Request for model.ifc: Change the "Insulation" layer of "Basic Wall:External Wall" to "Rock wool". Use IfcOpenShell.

First a look at what the model holds.

```python
import ifcopenshell
import ifcopenshell.util.element

model = ifcopenshell.open("model.ifc")
print(model.schema)
for layer_set in model.by_type("IfcMaterialLayerSet"):
    if layer_set.LayerSetName == "Basic Wall:External Wall":
        for layer in layer_set.MaterialLayers:
            print(layer.id(), layer.Material and layer.Material.Name, layer.LayerThickness, sep=" | ")
        print(len(ifcopenshell.util.element.get_elements_by_material(model, layer_set)), "elements and types use it")
print(sorted(m.Name for m in model.by_type("IfcMaterial") if m.Name)[:60])
```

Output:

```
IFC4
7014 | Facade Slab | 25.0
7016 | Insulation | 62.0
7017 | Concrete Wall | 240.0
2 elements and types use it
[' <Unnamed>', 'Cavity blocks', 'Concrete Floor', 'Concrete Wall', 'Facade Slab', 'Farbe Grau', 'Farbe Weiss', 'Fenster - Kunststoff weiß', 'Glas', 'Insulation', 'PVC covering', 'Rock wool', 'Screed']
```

```python
import ifcopenshell
import ifcopenshell.api.material

model = ifcopenshell.open("model.ifc")

layer_set = next(s for s in model.by_type("IfcMaterialLayerSet") if s.LayerSetName == "Basic Wall:External Wall")
layer = next(l for l in layer_set.MaterialLayers if l.Material and l.Material.Name == "Insulation")
material = next(m for m in model.by_type("IfcMaterial") if m.Name == "Rock wool")

# Point this one layer at the other material; renaming the old one would change it everywhere.
ifcopenshell.api.material.edit_layer(model, layer=layer, attributes={}, material=material)

print([l.Material.Name if l.Material else None for l in layer_set.MaterialLayers])

model.write("model_v2.ifc")
```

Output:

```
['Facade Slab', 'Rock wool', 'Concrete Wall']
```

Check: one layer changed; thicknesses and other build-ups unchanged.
